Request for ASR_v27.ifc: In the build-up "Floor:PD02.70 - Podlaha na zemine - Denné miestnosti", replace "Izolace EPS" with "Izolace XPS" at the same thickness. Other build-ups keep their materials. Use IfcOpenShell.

First a look at what the model holds.

```python
import ifcopenshell
import ifcopenshell.util.element

model = ifcopenshell.open("ASR_v27.ifc")
print(model.schema)
for layer_set in model.by_type("IfcMaterialLayerSet"):
    if layer_set.LayerSetName == "Floor:PD02.70 - Podlaha na zemine - Denné miestnosti":
        for layer in layer_set.MaterialLayers:
            print(layer.id(), layer.Material and layer.Material.Name, layer.LayerThickness, sep=" | ")
        print(len(ifcopenshell.util.element.get_elements_by_material(model, layer_set)), "elements and types use it")
print(sorted(m.Name for m in model.by_type("IfcMaterial") if m.Name)[:60])
```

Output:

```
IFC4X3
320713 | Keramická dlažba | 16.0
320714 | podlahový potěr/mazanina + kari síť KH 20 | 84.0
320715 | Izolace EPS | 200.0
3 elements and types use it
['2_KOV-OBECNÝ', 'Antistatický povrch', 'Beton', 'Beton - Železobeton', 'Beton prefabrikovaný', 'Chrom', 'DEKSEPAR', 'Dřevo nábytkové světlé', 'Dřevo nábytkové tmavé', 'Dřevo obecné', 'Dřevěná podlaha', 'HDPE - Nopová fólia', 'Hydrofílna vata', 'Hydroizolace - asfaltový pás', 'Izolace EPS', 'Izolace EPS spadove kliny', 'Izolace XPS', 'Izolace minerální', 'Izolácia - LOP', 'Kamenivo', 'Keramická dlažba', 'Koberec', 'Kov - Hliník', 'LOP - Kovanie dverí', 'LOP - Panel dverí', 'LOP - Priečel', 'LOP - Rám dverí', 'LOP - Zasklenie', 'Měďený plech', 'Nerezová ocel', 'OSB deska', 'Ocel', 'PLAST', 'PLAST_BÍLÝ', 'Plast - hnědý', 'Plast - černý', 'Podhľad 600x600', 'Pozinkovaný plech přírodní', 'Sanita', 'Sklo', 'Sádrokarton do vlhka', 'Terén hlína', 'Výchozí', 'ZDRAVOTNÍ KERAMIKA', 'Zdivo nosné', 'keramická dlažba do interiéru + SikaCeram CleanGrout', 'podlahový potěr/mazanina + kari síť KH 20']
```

```python
import ifcopenshell
import ifcopenshell.api.material

model = ifcopenshell.open("ASR_v27.ifc")

layer_set = next(s for s in model.by_type("IfcMaterialLayerSet") if s.LayerSetName == "Floor:PD02.70 - Podlaha na zemine - Denné miestnosti")
layer = next(l for l in layer_set.MaterialLayers if l.Material and l.Material.Name == "Izolace EPS")
material = next(m for m in model.by_type("IfcMaterial") if m.Name == "Izolace XPS")

# Point this one layer at the other material; renaming the old one would change it everywhere.
ifcopenshell.api.material.edit_layer(model, layer=layer, attributes={"Name": material.Name}, material=material)

print([l.Material.Name if l.Material else None for l in layer_set.MaterialLayers])

model.write("ASR_v27_rev.ifc")
```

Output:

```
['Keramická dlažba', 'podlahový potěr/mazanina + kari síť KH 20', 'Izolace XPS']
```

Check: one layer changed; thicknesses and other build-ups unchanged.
